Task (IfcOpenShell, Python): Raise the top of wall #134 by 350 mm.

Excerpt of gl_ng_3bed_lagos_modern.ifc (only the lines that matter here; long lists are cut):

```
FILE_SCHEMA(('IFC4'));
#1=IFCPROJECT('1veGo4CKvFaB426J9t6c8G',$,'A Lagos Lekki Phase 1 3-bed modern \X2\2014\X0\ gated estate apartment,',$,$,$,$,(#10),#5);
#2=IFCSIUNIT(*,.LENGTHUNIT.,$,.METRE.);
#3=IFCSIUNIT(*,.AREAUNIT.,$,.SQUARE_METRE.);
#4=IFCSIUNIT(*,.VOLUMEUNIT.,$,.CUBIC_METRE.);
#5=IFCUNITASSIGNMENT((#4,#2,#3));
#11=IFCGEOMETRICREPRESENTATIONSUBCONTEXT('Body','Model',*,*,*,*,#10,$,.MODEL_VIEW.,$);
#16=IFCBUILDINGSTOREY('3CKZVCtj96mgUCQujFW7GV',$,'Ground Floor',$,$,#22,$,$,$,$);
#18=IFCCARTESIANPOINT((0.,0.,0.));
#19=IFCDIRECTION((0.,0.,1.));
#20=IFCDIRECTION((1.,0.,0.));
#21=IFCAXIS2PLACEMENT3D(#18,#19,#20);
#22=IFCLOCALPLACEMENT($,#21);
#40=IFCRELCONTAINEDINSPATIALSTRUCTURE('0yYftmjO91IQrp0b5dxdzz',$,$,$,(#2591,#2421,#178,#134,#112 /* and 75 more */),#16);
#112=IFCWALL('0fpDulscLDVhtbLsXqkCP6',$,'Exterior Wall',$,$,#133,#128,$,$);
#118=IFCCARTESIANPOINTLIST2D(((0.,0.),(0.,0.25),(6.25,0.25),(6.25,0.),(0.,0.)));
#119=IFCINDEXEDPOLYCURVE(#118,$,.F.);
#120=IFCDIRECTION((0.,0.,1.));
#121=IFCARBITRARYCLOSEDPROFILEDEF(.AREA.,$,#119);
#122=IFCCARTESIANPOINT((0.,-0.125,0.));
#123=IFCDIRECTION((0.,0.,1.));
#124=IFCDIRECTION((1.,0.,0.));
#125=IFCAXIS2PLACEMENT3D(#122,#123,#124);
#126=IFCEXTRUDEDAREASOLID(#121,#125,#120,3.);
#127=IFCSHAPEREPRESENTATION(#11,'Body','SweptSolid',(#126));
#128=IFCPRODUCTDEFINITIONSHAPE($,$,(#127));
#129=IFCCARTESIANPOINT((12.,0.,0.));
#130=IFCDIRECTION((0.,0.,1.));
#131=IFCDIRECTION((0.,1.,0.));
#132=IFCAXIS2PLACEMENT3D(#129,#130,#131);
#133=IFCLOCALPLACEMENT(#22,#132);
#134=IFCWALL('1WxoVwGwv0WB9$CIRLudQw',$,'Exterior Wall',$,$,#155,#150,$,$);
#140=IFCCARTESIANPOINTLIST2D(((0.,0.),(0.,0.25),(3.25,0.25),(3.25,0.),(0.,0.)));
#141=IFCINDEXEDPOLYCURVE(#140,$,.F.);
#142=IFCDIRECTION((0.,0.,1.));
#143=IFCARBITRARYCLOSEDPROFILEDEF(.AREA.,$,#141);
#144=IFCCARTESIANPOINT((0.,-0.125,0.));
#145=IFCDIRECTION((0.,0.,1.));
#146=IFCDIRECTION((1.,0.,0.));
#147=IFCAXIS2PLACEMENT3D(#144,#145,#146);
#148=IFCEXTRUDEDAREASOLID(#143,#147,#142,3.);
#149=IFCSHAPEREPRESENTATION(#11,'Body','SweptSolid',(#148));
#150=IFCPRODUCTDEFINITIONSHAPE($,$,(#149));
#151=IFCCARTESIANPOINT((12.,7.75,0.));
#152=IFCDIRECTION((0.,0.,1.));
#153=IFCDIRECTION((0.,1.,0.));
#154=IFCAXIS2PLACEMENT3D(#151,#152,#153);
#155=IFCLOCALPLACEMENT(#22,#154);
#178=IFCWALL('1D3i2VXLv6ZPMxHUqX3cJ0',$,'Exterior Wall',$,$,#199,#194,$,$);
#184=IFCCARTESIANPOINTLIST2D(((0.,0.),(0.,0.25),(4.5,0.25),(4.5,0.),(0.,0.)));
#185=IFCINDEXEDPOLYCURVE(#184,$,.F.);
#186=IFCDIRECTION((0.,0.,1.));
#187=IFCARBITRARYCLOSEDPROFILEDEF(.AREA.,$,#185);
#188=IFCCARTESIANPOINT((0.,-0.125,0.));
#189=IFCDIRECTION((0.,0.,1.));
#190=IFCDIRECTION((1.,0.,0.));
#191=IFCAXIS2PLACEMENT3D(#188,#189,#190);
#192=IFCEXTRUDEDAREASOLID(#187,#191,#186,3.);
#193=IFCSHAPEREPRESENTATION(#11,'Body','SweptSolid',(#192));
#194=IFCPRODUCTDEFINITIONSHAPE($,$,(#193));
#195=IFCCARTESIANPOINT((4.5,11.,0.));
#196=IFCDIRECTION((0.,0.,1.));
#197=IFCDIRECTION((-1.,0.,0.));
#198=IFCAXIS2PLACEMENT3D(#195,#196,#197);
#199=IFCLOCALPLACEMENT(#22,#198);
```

```python
import ifcopenshell
import ifcopenshell.geom
import ifcopenshell.util.representation
import ifcopenshell.util.shape
import ifcopenshell.util.unit

model = ifcopenshell.open("gl_ng_3bed_lagos_modern.ifc")
unit_scale = ifcopenshell.util.unit.calculate_unit_scale(model)
settings = ifcopenshell.geom.settings()


def volume(element):
    """Net volume in cubic metres, openings subtracted."""
    shape = ifcopenshell.geom.create_shape(settings, element)
    return ifcopenshell.util.shape.get_volume(shape.geometry)


wall = model.by_guid("1WxoVwGwv0WB9$CIRLudQw")
before = volume(wall)

body = ifcopenshell.util.representation.get_representation(wall, "Model", "Body")
solid = body.Items[0]
old_height = solid.Depth
solid.Depth += 0.35 / unit_scale
after = volume(wall)

print(f"height {old_height:g} -> {solid.Depth:g}, volume {before:.3f} -> {after:.3f} m3")

model.write("gl_ng_3bed_lagos_modern_updated.ifc")
```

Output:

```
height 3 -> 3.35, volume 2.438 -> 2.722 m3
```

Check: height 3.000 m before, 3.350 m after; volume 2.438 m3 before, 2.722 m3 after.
